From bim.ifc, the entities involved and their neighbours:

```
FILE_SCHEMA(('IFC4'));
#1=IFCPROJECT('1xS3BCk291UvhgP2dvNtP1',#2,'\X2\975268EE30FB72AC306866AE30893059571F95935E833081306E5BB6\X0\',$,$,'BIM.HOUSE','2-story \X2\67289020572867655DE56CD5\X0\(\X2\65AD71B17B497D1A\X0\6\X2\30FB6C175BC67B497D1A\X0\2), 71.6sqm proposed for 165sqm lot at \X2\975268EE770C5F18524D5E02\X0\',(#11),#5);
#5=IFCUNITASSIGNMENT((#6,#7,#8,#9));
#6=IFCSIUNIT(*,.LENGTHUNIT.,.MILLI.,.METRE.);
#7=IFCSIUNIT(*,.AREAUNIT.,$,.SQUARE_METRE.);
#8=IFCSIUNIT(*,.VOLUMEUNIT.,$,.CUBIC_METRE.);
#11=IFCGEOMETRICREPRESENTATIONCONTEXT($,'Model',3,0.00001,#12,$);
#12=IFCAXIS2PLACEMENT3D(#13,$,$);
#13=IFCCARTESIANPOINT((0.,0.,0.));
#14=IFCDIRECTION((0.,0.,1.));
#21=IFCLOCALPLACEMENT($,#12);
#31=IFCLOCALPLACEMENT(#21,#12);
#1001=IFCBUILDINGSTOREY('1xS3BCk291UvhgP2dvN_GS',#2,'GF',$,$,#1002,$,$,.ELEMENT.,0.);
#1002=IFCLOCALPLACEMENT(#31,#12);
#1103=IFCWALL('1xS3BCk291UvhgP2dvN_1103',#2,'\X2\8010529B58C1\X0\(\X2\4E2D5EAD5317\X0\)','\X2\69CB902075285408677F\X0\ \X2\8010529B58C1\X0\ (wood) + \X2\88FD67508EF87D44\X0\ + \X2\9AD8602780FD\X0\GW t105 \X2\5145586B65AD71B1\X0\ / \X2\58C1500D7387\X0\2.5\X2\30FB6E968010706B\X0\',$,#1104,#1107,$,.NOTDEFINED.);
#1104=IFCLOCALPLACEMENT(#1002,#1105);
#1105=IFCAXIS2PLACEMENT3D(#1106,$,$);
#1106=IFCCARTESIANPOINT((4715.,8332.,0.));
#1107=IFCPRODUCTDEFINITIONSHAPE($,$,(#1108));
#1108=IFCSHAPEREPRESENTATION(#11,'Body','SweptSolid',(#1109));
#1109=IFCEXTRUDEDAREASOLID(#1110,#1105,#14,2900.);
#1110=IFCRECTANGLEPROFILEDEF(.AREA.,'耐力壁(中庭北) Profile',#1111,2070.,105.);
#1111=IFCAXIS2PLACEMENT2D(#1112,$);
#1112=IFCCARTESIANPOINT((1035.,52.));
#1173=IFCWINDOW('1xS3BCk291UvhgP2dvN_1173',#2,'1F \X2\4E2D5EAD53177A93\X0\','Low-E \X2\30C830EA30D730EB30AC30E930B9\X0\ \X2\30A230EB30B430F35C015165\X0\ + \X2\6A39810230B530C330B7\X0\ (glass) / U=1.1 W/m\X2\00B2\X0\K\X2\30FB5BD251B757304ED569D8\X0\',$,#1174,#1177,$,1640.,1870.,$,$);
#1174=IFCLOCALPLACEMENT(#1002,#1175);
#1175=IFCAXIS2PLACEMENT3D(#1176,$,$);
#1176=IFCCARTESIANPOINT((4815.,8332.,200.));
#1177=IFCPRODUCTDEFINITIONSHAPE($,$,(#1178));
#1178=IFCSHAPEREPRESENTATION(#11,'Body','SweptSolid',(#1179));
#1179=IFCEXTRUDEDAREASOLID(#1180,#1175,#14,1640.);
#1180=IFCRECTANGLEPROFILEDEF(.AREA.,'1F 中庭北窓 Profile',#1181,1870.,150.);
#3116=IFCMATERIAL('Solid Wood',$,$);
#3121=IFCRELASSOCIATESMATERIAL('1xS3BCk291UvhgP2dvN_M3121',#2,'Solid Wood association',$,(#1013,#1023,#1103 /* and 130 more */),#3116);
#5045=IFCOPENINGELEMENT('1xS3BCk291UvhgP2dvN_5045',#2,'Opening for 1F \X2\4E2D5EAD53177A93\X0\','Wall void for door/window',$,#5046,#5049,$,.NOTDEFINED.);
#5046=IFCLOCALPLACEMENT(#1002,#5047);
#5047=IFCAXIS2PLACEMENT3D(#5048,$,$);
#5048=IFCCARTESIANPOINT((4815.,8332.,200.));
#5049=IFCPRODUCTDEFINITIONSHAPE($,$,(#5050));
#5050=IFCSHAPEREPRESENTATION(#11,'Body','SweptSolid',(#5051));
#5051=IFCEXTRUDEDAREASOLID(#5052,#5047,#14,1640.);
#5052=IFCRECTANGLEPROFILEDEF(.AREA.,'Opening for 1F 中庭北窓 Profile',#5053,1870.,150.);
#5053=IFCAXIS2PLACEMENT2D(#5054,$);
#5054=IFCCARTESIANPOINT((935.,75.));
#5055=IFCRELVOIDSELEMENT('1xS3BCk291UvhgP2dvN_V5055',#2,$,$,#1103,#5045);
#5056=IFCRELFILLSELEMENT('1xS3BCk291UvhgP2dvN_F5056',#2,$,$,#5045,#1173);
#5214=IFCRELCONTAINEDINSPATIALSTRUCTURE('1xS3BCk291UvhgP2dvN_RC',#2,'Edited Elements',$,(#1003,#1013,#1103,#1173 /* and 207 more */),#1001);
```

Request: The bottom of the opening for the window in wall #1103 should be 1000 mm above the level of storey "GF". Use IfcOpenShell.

```python
import numpy as np
import ifcopenshell
import ifcopenshell.api.geometry
import ifcopenshell.geom
import ifcopenshell.util.element
import ifcopenshell.util.placement
import ifcopenshell.util.shape
import ifcopenshell.util.unit

model = ifcopenshell.open("bim.ifc")
unit_scale = ifcopenshell.util.unit.calculate_unit_scale(model)

window = model.by_guid("1xS3BCk291UvhgP2dvN_1173")
opening = window.FillsVoids[0].RelatingOpeningElement
storey = ifcopenshell.util.element.get_container(window, ifc_class="IfcBuildingStorey")
level = ifcopenshell.util.placement.get_local_placement(storey.ObjectPlacement)[2, 3]

# The opening's origin need not be at the sill, so measure its lowest point.
shape = ifcopenshell.geom.create_shape(ifcopenshell.geom.settings(), opening)
bottom = ifcopenshell.util.shape.get_shape_bottom_elevation(shape, shape.geometry) / unit_scale
dz = level + 1 / unit_scale - bottom

shift = np.array([0.0, 0.0, dz])
# The window is not placed relative to its opening, so move both.
for product in (opening, window):
    matrix = ifcopenshell.util.placement.get_local_placement(product.ObjectPlacement)
    matrix[:3, 3] += shift
    ifcopenshell.api.geometry.edit_object_placement(model, product=product, matrix=matrix, is_si=False)

print(f"moved by {dz * unit_scale:+.3f} m")

model.write("bim_edited.ifc")
```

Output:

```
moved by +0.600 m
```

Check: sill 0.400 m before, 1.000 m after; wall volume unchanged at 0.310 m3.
